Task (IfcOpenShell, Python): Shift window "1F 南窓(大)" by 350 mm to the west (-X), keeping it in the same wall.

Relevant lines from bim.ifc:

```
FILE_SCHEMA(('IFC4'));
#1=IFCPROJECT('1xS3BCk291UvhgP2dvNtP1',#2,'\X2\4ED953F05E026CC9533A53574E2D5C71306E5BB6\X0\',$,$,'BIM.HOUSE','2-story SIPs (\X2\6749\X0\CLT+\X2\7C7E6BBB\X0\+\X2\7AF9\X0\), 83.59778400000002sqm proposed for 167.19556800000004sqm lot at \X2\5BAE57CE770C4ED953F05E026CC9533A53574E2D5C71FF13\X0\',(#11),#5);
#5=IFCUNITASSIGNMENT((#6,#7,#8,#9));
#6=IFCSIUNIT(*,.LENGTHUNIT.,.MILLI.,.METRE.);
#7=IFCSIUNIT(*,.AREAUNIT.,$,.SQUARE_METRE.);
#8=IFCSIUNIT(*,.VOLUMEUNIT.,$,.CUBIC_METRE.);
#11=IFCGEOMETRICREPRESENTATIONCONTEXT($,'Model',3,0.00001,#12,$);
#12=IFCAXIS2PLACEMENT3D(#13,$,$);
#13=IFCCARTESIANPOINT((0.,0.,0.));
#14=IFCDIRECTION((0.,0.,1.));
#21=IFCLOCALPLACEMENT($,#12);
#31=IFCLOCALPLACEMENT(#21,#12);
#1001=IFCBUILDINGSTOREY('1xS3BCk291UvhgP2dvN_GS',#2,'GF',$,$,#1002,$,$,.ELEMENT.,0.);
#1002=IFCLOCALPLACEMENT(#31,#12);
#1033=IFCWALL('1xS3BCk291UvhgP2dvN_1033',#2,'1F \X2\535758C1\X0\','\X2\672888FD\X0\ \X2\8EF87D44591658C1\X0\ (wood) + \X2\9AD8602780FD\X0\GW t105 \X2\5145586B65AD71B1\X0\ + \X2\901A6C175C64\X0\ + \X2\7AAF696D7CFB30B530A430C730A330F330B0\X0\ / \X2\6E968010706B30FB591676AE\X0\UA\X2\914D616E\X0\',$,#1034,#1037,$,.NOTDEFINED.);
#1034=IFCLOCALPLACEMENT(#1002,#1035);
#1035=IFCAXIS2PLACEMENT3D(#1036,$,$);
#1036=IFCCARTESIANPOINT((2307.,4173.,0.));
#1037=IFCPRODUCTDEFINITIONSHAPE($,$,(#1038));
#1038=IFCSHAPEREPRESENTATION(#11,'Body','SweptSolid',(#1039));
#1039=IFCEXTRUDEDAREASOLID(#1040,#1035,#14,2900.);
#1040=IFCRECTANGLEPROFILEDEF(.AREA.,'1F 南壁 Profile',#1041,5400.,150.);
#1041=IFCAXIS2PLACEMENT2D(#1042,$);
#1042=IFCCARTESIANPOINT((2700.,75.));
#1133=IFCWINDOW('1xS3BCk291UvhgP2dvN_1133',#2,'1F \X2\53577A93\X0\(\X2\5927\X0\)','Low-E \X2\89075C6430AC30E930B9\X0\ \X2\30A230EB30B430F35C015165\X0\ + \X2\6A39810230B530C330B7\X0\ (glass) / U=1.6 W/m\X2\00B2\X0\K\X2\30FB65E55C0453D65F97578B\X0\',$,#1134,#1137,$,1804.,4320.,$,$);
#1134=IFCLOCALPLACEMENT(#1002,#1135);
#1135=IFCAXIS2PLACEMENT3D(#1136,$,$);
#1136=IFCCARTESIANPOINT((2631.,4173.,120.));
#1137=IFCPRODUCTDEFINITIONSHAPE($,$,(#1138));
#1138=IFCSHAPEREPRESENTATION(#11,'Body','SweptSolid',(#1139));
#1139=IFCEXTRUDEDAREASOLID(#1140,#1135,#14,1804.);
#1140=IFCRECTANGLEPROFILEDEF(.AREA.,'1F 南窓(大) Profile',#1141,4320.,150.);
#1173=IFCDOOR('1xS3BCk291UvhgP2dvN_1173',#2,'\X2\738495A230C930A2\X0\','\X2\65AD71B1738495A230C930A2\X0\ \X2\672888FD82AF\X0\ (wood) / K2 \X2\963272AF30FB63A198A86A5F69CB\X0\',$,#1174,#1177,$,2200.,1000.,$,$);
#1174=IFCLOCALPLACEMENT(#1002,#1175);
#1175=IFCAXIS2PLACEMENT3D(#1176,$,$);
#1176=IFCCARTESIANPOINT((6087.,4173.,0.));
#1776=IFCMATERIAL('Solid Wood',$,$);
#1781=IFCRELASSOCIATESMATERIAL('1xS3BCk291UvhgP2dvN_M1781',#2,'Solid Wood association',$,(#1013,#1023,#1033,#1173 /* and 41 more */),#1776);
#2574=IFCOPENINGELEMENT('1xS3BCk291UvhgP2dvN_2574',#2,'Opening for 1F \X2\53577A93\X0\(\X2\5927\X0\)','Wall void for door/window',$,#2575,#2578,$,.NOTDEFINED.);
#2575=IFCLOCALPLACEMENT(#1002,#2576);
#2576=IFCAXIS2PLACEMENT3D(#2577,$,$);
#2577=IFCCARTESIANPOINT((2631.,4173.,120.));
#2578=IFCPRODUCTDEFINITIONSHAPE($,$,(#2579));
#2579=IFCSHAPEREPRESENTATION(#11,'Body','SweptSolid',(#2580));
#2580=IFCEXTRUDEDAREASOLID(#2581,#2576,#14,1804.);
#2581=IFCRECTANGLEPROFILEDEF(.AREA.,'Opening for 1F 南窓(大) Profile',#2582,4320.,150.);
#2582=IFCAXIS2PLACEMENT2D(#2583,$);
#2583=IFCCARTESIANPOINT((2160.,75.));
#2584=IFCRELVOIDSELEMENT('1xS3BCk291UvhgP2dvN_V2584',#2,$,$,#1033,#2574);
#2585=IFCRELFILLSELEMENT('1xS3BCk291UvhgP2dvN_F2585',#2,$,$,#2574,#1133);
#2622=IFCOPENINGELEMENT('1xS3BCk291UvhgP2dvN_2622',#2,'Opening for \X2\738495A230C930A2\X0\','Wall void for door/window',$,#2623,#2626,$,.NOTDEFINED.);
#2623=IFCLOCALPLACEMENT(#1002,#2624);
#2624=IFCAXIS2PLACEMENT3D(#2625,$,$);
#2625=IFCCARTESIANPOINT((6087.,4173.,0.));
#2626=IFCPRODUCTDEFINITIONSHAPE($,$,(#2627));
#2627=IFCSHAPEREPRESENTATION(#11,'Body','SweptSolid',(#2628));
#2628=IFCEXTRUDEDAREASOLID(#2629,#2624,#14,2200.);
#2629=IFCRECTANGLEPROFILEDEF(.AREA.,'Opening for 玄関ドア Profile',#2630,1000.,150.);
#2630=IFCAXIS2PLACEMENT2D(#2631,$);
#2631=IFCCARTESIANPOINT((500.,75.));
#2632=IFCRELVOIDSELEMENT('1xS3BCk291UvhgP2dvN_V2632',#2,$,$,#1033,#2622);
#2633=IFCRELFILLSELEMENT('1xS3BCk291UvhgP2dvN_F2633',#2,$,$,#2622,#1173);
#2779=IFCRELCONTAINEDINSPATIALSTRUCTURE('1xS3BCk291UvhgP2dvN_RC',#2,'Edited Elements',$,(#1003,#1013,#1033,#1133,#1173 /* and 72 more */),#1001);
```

```python
import ifcopenshell
import ifcopenshell.api.geometry
import ifcopenshell.util.placement

model = ifcopenshell.open("bim.ifc")

window = model.by_id(1133)
opening = window.FillsVoids[0].RelatingOpeningElement
wall = opening.VoidsElements[0].RelatingBuildingElement

wall_matrix = ifcopenshell.util.placement.get_local_placement(wall.ObjectPlacement)
shift = wall_matrix[:3, 0] * -350.0
before = ifcopenshell.util.placement.get_local_placement(window.ObjectPlacement)[:3, 3].copy()

# The window is not placed relative to its opening, so move both.
for product in (opening, window):
    matrix = ifcopenshell.util.placement.get_local_placement(product.ObjectPlacement)
    matrix[:3, 3] += shift
    ifcopenshell.api.geometry.edit_object_placement(model, product=product, matrix=matrix, is_si=False)

after = ifcopenshell.util.placement.get_local_placement(window.ObjectPlacement)[:3, 3]
print("window moved by", (after - before).round(3) + 0.0)

model.write("bim_edited.ifc")
```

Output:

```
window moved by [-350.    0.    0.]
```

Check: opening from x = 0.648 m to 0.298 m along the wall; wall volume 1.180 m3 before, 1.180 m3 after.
